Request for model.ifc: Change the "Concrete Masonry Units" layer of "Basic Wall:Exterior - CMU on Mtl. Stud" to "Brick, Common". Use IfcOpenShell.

First a look at what the model holds.

```python
import ifcopenshell
import ifcopenshell.util.element

model = ifcopenshell.open("model.ifc")
print(model.schema)
for layer_set in model.by_type("IfcMaterialLayerSet"):
    if layer_set.LayerSetName == "Basic Wall:Exterior - CMU on Mtl. Stud":
        for layer in layer_set.MaterialLayers:
            print(layer.id(), layer.Material and layer.Material.Name, layer.LayerThickness, sep=" | ")
        print(len(ifcopenshell.util.element.get_elements_by_material(model, layer_set)), "elements and types use it")
print(sorted(m.Name for m in model.by_type("IfcMaterial") if m.Name)[:60])
```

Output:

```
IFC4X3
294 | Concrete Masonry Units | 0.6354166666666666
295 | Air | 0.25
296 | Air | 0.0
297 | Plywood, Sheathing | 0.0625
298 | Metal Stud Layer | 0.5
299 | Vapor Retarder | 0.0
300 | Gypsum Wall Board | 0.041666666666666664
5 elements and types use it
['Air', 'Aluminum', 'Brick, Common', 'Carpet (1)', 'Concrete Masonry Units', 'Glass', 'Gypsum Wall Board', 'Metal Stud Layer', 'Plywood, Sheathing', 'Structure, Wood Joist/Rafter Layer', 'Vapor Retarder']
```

```python
import ifcopenshell
import ifcopenshell.api.material

model = ifcopenshell.open("model.ifc")

layer_set = next(s for s in model.by_type("IfcMaterialLayerSet") if s.LayerSetName == "Basic Wall:Exterior - CMU on Mtl. Stud")
layer = next(l for l in layer_set.MaterialLayers if l.Material and l.Material.Name == "Concrete Masonry Units")
material = next(m for m in model.by_type("IfcMaterial") if m.Name == "Brick, Common")

# Point this one layer at the other material; renaming the old one would change it everywhere.
ifcopenshell.api.material.edit_layer(model, layer=layer, attributes={"Name": material.Name}, material=material)

print([l.Material.Name if l.Material else None for l in layer_set.MaterialLayers])

model.write("model_rev.ifc")
```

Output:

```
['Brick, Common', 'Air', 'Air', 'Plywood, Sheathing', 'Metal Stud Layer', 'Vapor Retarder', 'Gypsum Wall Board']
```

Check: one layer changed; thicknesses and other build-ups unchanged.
